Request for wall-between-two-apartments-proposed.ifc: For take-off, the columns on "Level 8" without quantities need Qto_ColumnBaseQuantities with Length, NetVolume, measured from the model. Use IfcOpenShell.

First a look at what the model holds.

```python
import ifcopenshell
import ifcopenshell.util.element
import ifcopenshell.util.unit

model = ifcopenshell.open("wall-between-two-apartments-proposed.ifc")
print(model.schema)
for unit_type in ("LENGTHUNIT", "AREAUNIT", "VOLUMEUNIT"):
    print(unit_type, ifcopenshell.util.unit.calculate_unit_scale(model, unit_type))
storey = next(s for s in model.by_type("IfcBuildingStorey") if s.Name == "Level 8")
columns = [e for e in ifcopenshell.util.element.get_decomposition(storey) if e.is_a("IfcColumn")]
for e in sorted(columns, key=lambda e: e.id()):
    print(e.id(), e.is_a(), e.Name, list(ifcopenshell.util.element.get_psets(e, qtos_only=True)), sep=" | ")
```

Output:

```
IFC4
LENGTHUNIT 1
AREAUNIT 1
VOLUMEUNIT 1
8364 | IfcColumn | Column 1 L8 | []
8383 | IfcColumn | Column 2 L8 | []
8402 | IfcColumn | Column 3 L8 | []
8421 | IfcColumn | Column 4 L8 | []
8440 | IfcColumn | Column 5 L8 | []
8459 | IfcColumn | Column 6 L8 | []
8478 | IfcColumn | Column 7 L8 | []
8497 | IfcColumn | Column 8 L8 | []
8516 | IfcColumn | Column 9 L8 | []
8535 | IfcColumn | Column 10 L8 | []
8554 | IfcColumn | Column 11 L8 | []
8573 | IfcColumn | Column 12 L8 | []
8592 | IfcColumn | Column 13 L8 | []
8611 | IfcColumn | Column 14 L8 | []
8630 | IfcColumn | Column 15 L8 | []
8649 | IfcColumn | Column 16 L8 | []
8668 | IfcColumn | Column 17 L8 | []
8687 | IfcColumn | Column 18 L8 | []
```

```python
import ifcopenshell
import ifcopenshell.api.pset
import ifcopenshell.geom
import ifcopenshell.util.element
import ifcopenshell.util.shape
import ifcopenshell.util.unit

model = ifcopenshell.open("wall-between-two-apartments-proposed.ifc")
unit_scale = ifcopenshell.util.unit.calculate_unit_scale(model)
volume_scale = ifcopenshell.util.unit.calculate_unit_scale(model, "VOLUMEUNIT")
settings = ifcopenshell.geom.settings()

storey = next(s for s in model.by_type("IfcBuildingStorey") if s.Name == "Level 8")
columns = [e for e in ifcopenshell.util.element.get_decomposition(storey) if e.is_a("IfcColumn")]

for e in sorted(columns, key=lambda e: e.id()):
    if ifcopenshell.util.element.get_psets(e, qtos_only=True, should_inherit=False):
        continue
    # Geometry comes back in metres, in the element's own axes.
    shape = ifcopenshell.geom.create_shape(settings, e)
    values = {
        "Length": ifcopenshell.util.shape.get_z(shape.geometry) / unit_scale,
        "NetVolume": ifcopenshell.util.shape.get_volume(shape.geometry) / volume_scale,
    }
    qto = ifcopenshell.api.pset.add_qto(model, product=e, name="Qto_ColumnBaseQuantities")
    ifcopenshell.api.pset.edit_qto(model, qto=qto, properties=values)
    print(e.id(), {k: round(v, 3) for k, v in values.items()})

model.write("wall-between-two-apartments-proposed_updated.ifc")
```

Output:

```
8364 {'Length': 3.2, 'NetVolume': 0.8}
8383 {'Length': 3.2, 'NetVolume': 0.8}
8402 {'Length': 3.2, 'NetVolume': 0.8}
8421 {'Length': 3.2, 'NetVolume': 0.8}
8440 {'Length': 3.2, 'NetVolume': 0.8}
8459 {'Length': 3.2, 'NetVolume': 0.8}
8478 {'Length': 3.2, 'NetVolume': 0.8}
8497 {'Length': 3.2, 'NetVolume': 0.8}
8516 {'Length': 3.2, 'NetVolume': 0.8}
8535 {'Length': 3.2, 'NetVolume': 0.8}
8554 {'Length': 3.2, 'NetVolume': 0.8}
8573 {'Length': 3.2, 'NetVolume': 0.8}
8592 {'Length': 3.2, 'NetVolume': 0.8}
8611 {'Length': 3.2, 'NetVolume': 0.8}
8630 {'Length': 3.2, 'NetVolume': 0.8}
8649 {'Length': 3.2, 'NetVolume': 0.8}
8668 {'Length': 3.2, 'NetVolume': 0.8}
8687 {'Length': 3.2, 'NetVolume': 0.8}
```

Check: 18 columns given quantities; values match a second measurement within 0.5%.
